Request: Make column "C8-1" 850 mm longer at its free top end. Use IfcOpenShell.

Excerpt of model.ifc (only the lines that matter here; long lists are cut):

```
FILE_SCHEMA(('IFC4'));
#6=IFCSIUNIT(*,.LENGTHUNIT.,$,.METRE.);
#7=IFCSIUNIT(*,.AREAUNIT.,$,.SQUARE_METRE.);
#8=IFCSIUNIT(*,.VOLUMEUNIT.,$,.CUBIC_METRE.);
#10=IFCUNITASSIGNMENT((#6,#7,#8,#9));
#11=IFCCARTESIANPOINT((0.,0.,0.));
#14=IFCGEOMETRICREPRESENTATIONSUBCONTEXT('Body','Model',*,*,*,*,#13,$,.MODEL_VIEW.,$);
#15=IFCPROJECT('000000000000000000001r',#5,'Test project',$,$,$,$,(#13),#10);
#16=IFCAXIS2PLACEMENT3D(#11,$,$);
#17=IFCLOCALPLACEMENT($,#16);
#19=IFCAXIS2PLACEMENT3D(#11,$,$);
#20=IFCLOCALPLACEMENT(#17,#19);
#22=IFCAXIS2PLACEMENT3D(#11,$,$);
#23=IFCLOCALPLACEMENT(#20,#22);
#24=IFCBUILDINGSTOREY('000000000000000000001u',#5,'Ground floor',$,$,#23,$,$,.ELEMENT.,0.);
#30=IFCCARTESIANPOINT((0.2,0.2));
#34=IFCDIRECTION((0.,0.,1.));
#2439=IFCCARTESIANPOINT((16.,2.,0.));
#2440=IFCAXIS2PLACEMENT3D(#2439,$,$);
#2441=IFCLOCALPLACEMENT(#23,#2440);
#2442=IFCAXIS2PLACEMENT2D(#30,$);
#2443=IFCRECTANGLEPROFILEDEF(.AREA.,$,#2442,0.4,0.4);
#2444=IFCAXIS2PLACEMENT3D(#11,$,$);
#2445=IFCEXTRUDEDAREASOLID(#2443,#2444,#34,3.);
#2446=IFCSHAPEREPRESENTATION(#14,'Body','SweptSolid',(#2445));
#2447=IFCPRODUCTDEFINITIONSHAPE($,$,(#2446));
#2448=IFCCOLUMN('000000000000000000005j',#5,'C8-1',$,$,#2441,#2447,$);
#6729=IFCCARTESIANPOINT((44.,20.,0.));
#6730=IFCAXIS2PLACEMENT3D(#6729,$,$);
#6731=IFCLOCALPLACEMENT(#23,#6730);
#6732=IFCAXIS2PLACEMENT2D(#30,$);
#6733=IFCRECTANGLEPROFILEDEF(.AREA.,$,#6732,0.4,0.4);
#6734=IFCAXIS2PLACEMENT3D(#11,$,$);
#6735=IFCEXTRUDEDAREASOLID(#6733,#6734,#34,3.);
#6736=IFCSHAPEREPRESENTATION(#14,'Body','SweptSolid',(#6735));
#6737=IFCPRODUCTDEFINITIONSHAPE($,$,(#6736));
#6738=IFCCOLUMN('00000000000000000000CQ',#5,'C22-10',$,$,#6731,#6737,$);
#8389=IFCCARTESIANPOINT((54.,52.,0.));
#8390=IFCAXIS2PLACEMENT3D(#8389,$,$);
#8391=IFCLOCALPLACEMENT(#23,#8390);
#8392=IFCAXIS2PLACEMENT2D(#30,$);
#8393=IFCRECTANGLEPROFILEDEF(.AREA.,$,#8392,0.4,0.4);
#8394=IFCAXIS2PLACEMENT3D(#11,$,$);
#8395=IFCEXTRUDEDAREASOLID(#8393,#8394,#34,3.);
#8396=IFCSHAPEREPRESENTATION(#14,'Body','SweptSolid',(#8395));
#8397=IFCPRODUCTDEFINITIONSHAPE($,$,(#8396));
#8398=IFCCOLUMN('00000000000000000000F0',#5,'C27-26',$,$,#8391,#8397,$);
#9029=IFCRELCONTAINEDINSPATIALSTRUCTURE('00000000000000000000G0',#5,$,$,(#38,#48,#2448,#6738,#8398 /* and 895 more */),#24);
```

```python
import ifcopenshell
import ifcopenshell.util.representation
import ifcopenshell.util.unit

model = ifcopenshell.open("model.ifc")
unit_scale = ifcopenshell.util.unit.calculate_unit_scale(model)

member = model.by_id(2448)
change = 0.85 / unit_scale

# The extrusion runs towards the end named, so only its depth changes.
body = ifcopenshell.util.representation.get_representation(member, "Model", "Body")
solid = body.Items[0]
old_length = solid.Depth
solid.Depth += change

print(f"length {old_length:g} -> {solid.Depth:g}")

model.write("model-out.ifc")
```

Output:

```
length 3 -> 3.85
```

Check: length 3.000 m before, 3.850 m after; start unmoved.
